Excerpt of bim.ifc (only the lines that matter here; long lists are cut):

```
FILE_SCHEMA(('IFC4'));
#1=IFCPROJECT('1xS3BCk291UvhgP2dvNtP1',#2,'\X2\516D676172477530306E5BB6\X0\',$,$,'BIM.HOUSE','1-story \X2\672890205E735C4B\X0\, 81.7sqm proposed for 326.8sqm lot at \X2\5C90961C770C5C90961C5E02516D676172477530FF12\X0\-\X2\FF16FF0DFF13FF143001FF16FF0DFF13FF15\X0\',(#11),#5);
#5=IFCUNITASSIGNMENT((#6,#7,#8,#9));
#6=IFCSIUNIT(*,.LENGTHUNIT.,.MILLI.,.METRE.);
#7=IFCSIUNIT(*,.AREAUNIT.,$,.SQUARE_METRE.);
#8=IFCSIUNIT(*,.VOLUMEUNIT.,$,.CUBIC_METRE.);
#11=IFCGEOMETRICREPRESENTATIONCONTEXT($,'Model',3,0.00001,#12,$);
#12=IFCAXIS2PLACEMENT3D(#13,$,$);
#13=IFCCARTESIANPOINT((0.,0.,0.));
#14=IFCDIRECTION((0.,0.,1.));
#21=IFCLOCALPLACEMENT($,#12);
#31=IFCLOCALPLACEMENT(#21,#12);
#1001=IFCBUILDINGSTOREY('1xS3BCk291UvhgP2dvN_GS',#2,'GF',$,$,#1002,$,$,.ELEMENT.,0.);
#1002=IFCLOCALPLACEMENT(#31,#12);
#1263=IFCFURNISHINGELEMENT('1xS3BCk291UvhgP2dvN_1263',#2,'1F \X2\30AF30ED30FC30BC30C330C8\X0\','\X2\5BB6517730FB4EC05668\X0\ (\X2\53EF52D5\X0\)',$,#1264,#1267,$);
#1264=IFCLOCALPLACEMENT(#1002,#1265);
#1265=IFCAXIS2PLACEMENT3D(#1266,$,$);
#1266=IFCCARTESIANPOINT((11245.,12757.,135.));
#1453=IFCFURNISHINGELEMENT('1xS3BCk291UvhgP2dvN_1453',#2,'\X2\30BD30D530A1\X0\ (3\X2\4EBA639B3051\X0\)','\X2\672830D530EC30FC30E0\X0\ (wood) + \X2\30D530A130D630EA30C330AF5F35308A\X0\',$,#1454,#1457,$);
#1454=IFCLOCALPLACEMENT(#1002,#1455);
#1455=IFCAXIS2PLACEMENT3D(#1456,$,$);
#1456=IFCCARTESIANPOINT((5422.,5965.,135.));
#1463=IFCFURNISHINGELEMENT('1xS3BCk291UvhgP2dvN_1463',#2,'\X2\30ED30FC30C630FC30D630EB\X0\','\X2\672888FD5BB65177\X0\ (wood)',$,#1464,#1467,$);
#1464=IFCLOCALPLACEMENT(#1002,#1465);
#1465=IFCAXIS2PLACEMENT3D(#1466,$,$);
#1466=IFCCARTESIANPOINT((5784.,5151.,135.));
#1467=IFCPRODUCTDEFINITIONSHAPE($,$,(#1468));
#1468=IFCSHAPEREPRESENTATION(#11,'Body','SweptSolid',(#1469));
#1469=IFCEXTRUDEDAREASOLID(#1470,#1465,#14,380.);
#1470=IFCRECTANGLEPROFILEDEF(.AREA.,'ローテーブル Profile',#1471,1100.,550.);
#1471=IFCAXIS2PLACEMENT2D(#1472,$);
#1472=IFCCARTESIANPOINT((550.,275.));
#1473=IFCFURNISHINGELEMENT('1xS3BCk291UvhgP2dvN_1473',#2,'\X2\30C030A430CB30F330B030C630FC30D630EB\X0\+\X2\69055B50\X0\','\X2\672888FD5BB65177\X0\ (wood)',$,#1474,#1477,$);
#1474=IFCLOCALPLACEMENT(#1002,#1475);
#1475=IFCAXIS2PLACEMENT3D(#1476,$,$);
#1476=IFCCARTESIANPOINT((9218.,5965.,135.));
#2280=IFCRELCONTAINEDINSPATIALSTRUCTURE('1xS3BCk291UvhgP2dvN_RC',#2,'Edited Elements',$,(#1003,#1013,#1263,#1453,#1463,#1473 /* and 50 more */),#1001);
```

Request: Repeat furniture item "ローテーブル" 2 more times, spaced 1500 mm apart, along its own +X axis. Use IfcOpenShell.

```python
import ifcopenshell
import ifcopenshell.api.geometry
import ifcopenshell.api.root
import ifcopenshell.util.element
import ifcopenshell.util.placement
import ifcopenshell.util.unit

model = ifcopenshell.open("bim.ifc")
unit_scale = ifcopenshell.util.unit.calculate_unit_scale(model)


def reuse_history(source, copy):
    """copy_class also copies each property set's owner history, people and application; keep the originals."""
    for rel in copy.IsDefinedBy:
        if rel.is_a("IfcRelDefinesByProperties") and (history := rel.RelatingPropertyDefinition.OwnerHistory):
            rel.RelatingPropertyDefinition.OwnerHistory = source.OwnerHistory
            ifcopenshell.util.element.remove_deep2(model, history)


source = model.by_guid("1xS3BCk291UvhgP2dvN_1463")
base = ifcopenshell.util.placement.get_local_placement(source.ObjectPlacement)
step = base[:3, 0] * 1.5 / unit_scale

for i in range(1, 3):
    copy = ifcopenshell.api.root.copy_class(model, product=source)
    copy.Representation = ifcopenshell.util.element.copy_deep(
        model, source.Representation, exclude=["IfcGeometricRepresentationContext", "IfcRepresentationMap"]
    )
    reuse_history(source, copy)
    matrix = base.copy()
    matrix[:3, 3] += i * step
    print("added at", matrix[:3, 3].round(3) + 0.0)
    ifcopenshell.api.geometry.edit_object_placement(model, product=copy, matrix=matrix, is_si=False)

model.write("bim-out.ifc")
```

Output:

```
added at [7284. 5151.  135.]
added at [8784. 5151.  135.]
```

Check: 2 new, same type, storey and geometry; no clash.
